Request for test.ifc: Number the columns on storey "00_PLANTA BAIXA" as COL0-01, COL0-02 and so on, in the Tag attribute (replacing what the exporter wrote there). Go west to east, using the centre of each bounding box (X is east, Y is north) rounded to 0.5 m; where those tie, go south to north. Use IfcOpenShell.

First a look at what the model holds.

```python
import ifcopenshell
import ifcopenshell.util.element
import ifcopenshell.util.placement

model = ifcopenshell.open("test.ifc")
print(model.schema)
storey = next(s for s in model.by_type("IfcBuildingStorey") if s.Name == "00_PLANTA BAIXA")
columns = [e for e in ifcopenshell.util.element.get_decomposition(storey) if e.is_a("IfcColumn")]
for e in sorted(columns, key=lambda e: e.id()):
    origin = ifcopenshell.util.placement.get_local_placement(e.ObjectPlacement)[:3, 3]
    print(e.id(), e.Tag, e.Name, origin.round(2) + 0.0, sep=" | ")
```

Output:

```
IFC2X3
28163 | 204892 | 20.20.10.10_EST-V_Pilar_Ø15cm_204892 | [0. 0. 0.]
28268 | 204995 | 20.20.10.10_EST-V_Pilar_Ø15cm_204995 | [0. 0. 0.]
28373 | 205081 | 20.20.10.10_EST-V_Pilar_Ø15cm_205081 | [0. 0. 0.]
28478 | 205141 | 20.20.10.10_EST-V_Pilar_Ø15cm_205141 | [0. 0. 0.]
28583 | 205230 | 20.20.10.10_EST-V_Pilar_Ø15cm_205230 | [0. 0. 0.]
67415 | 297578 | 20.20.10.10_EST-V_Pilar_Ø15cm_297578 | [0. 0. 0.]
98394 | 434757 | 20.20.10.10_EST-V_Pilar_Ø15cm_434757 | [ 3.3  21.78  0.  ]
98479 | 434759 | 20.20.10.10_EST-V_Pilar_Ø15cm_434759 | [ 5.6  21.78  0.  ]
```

```python
import ifcopenshell
import ifcopenshell.geom
import ifcopenshell.util.element
import ifcopenshell.util.shape

model = ifcopenshell.open("test.ifc")
settings = ifcopenshell.geom.settings()
settings.set("use-world-coords", True)


def centre(element):
    shape = ifcopenshell.geom.create_shape(settings, element)
    return ifcopenshell.util.shape.get_bbox_centroid(shape.geometry)


storey = next(s for s in model.by_type("IfcBuildingStorey") if s.Name == "00_PLANTA BAIXA")
columns = [e for e in ifcopenshell.util.element.get_decomposition(storey) if e.is_a("IfcColumn")]

# Insertion points can sit at a corner or the storey origin, so sort by the geometry (in metres).
centres = {e: centre(e) for e in columns}
columns.sort(key=lambda e: (round(centres[e][0] / 0.5), centres[e][1]))

for i, e in enumerate(columns, start=1):
    number = f"COL0-{i:02d}"
    e.Tag = number
    print(e.id(), number)

model.write("test_rev.ifc")
```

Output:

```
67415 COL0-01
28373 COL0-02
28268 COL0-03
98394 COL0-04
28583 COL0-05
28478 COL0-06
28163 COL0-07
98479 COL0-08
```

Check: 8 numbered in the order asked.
